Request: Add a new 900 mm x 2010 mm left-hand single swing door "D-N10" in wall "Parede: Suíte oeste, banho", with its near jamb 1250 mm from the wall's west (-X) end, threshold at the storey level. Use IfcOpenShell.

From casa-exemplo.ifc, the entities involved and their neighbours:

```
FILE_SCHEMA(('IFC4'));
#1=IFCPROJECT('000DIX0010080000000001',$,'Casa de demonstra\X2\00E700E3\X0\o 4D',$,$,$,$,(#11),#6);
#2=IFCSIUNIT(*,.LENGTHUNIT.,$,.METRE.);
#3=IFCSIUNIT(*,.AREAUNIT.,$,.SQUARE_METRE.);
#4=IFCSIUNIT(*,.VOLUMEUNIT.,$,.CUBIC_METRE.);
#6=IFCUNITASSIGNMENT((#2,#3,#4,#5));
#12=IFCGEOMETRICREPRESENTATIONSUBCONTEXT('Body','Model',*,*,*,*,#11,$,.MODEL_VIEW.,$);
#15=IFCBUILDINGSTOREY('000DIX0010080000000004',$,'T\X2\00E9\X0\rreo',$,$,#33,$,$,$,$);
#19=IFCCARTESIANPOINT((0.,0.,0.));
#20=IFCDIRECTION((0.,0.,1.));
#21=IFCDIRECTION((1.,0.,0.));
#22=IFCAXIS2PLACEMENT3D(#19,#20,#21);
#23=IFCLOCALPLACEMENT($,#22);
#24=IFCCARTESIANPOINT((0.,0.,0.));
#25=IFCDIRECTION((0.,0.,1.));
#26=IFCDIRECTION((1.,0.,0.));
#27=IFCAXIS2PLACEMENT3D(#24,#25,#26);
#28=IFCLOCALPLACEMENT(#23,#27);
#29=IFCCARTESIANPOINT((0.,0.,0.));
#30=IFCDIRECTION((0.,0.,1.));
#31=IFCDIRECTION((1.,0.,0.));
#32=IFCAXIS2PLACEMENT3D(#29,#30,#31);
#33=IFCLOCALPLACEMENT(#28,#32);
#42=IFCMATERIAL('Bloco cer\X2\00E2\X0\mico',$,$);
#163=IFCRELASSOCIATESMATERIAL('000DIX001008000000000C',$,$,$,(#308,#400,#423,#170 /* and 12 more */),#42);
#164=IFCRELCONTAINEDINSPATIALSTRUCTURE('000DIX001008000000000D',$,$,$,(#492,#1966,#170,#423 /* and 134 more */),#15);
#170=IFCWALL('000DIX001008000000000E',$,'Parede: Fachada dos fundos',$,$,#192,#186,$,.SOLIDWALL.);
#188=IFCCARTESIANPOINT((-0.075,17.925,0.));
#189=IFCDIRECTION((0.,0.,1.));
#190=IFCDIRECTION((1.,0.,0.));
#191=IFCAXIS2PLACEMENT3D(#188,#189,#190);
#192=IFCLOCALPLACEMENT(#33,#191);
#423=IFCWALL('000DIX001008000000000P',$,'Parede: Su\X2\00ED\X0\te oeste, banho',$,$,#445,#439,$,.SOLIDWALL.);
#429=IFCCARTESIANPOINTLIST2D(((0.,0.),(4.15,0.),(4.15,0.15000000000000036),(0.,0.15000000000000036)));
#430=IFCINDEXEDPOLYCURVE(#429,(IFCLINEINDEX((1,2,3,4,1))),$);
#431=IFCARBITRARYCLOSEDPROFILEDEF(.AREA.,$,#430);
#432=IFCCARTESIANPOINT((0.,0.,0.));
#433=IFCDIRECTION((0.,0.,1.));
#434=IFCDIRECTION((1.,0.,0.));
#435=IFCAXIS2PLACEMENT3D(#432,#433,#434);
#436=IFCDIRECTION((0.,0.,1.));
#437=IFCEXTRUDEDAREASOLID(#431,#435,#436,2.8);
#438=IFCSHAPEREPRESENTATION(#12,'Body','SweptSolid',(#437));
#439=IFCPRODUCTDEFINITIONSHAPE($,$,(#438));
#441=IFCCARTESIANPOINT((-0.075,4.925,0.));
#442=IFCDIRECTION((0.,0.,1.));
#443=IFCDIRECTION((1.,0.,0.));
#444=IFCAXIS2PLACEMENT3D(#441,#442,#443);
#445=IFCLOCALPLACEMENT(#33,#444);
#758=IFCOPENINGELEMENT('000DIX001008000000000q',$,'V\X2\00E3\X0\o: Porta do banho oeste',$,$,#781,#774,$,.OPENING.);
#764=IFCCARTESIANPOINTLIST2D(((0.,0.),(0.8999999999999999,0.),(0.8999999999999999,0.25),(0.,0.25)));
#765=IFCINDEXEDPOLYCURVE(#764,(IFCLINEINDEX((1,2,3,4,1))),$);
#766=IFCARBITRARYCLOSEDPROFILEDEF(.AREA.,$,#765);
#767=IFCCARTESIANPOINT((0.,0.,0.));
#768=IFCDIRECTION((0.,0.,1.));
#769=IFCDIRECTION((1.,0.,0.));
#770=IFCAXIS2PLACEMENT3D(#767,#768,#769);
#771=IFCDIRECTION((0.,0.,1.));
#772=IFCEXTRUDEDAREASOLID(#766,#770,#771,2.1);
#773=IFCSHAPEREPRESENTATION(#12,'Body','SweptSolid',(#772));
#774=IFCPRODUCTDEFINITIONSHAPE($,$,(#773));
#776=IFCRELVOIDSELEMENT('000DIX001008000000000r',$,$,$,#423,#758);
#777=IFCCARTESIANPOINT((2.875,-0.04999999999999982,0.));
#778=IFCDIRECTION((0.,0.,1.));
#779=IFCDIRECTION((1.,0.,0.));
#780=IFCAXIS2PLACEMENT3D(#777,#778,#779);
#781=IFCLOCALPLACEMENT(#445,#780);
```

```python
import numpy as np
import ifcopenshell
import ifcopenshell.api.feature
import ifcopenshell.api.geometry
import ifcopenshell.api.root
import ifcopenshell.api.spatial
import ifcopenshell.geom
import ifcopenshell.util.element
import ifcopenshell.util.placement
import ifcopenshell.util.representation
import ifcopenshell.util.shape
import ifcopenshell.util.unit

model = ifcopenshell.open("casa-exemplo.ifc")
unit_scale = ifcopenshell.util.unit.calculate_unit_scale(model)
settings = ifcopenshell.geom.settings()


def volume(element):
    """Net volume in cubic metres, openings subtracted."""
    shape = ifcopenshell.geom.create_shape(settings, element)
    return ifcopenshell.util.shape.get_volume(shape.geometry)


wall = model.by_id(423)
storey = ifcopenshell.util.element.get_container(wall, ifc_class="IfcBuildingStorey")
context = ifcopenshell.util.representation.get_context(model, "Model", "Body", "MODEL_VIEW")
before = volume(wall)

width, height, from_end, sill = 0.9, 2.01, 1.25, 0.0  # metres

# The wall runs along its own X axis, and the end named is its -X end.
wall_shape = ifcopenshell.geom.create_shape(settings, wall)
x, y, z = ifcopenshell.util.shape.get_vertices(wall_shape.geometry).T
start = x.min() + from_end
face, thickness = float(y.min()), float(y.max() - y.min())
wall_matrix = ifcopenshell.util.placement.get_local_placement(wall.ObjectPlacement)
level = ifcopenshell.util.placement.get_local_placement(storey.ObjectPlacement)[2, 3]


def in_wall(x, y):
    """Placement at x, y metres in the wall's axes, at sill height."""
    matrix = wall_matrix.copy()
    matrix[:, 3] = wall_matrix @ np.array([x / unit_scale, y / unit_scale, 0.0, 1.0])
    matrix[2, 3] = level + sill / unit_scale
    return matrix


# Opening: a box that overshoots both wall faces by 50 mm.
opening = ifcopenshell.api.root.create_entity(model, ifc_class="IfcOpeningElement", predefined_type="OPENING")
box = ifcopenshell.api.geometry.add_wall_representation(
    model, context=context, length=width, height=height, thickness=thickness + 0.1
)
ifcopenshell.api.geometry.assign_representation(model, product=opening, representation=box)
ifcopenshell.api.geometry.edit_object_placement(model, product=opening, matrix=in_wall(start, face - 0.05), is_si=False)
ifcopenshell.api.feature.add_feature(model, feature=opening, element=wall)

door = ifcopenshell.api.root.create_entity(model, ifc_class="IfcDoor", name="D-N10", predefined_type="DOOR")
door.OverallWidth, door.OverallHeight = width / unit_scale, height / unit_scale
door.OperationType = "SINGLE_SWING_LEFT"
body = ifcopenshell.api.geometry.add_door_representation(
    model,
    context=context,
    overall_width=door.OverallWidth,
    overall_height=door.OverallHeight,
    operation_type="SINGLE_SWING_LEFT",
    lining_properties={"LiningDepth": thickness / unit_scale, "ThresholdDepth": thickness / unit_scale},
)
ifcopenshell.api.geometry.assign_representation(model, product=door, representation=body)
ifcopenshell.api.spatial.assign_container(model, products=[door], relating_structure=storey)
ifcopenshell.api.feature.add_filling(model, opening=opening, element=door)

# The lining spans the wall, so the door starts at the wall face.
ifcopenshell.api.geometry.edit_object_placement(model, product=door, matrix=in_wall(start, face), is_si=False)

after = volume(wall)

print(f"wall volume {before:.3f} -> {after:.3f} m3")

model.write("casa-exemplo-out.ifc")
```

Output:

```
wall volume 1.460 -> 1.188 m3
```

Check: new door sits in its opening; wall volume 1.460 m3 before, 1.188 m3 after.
